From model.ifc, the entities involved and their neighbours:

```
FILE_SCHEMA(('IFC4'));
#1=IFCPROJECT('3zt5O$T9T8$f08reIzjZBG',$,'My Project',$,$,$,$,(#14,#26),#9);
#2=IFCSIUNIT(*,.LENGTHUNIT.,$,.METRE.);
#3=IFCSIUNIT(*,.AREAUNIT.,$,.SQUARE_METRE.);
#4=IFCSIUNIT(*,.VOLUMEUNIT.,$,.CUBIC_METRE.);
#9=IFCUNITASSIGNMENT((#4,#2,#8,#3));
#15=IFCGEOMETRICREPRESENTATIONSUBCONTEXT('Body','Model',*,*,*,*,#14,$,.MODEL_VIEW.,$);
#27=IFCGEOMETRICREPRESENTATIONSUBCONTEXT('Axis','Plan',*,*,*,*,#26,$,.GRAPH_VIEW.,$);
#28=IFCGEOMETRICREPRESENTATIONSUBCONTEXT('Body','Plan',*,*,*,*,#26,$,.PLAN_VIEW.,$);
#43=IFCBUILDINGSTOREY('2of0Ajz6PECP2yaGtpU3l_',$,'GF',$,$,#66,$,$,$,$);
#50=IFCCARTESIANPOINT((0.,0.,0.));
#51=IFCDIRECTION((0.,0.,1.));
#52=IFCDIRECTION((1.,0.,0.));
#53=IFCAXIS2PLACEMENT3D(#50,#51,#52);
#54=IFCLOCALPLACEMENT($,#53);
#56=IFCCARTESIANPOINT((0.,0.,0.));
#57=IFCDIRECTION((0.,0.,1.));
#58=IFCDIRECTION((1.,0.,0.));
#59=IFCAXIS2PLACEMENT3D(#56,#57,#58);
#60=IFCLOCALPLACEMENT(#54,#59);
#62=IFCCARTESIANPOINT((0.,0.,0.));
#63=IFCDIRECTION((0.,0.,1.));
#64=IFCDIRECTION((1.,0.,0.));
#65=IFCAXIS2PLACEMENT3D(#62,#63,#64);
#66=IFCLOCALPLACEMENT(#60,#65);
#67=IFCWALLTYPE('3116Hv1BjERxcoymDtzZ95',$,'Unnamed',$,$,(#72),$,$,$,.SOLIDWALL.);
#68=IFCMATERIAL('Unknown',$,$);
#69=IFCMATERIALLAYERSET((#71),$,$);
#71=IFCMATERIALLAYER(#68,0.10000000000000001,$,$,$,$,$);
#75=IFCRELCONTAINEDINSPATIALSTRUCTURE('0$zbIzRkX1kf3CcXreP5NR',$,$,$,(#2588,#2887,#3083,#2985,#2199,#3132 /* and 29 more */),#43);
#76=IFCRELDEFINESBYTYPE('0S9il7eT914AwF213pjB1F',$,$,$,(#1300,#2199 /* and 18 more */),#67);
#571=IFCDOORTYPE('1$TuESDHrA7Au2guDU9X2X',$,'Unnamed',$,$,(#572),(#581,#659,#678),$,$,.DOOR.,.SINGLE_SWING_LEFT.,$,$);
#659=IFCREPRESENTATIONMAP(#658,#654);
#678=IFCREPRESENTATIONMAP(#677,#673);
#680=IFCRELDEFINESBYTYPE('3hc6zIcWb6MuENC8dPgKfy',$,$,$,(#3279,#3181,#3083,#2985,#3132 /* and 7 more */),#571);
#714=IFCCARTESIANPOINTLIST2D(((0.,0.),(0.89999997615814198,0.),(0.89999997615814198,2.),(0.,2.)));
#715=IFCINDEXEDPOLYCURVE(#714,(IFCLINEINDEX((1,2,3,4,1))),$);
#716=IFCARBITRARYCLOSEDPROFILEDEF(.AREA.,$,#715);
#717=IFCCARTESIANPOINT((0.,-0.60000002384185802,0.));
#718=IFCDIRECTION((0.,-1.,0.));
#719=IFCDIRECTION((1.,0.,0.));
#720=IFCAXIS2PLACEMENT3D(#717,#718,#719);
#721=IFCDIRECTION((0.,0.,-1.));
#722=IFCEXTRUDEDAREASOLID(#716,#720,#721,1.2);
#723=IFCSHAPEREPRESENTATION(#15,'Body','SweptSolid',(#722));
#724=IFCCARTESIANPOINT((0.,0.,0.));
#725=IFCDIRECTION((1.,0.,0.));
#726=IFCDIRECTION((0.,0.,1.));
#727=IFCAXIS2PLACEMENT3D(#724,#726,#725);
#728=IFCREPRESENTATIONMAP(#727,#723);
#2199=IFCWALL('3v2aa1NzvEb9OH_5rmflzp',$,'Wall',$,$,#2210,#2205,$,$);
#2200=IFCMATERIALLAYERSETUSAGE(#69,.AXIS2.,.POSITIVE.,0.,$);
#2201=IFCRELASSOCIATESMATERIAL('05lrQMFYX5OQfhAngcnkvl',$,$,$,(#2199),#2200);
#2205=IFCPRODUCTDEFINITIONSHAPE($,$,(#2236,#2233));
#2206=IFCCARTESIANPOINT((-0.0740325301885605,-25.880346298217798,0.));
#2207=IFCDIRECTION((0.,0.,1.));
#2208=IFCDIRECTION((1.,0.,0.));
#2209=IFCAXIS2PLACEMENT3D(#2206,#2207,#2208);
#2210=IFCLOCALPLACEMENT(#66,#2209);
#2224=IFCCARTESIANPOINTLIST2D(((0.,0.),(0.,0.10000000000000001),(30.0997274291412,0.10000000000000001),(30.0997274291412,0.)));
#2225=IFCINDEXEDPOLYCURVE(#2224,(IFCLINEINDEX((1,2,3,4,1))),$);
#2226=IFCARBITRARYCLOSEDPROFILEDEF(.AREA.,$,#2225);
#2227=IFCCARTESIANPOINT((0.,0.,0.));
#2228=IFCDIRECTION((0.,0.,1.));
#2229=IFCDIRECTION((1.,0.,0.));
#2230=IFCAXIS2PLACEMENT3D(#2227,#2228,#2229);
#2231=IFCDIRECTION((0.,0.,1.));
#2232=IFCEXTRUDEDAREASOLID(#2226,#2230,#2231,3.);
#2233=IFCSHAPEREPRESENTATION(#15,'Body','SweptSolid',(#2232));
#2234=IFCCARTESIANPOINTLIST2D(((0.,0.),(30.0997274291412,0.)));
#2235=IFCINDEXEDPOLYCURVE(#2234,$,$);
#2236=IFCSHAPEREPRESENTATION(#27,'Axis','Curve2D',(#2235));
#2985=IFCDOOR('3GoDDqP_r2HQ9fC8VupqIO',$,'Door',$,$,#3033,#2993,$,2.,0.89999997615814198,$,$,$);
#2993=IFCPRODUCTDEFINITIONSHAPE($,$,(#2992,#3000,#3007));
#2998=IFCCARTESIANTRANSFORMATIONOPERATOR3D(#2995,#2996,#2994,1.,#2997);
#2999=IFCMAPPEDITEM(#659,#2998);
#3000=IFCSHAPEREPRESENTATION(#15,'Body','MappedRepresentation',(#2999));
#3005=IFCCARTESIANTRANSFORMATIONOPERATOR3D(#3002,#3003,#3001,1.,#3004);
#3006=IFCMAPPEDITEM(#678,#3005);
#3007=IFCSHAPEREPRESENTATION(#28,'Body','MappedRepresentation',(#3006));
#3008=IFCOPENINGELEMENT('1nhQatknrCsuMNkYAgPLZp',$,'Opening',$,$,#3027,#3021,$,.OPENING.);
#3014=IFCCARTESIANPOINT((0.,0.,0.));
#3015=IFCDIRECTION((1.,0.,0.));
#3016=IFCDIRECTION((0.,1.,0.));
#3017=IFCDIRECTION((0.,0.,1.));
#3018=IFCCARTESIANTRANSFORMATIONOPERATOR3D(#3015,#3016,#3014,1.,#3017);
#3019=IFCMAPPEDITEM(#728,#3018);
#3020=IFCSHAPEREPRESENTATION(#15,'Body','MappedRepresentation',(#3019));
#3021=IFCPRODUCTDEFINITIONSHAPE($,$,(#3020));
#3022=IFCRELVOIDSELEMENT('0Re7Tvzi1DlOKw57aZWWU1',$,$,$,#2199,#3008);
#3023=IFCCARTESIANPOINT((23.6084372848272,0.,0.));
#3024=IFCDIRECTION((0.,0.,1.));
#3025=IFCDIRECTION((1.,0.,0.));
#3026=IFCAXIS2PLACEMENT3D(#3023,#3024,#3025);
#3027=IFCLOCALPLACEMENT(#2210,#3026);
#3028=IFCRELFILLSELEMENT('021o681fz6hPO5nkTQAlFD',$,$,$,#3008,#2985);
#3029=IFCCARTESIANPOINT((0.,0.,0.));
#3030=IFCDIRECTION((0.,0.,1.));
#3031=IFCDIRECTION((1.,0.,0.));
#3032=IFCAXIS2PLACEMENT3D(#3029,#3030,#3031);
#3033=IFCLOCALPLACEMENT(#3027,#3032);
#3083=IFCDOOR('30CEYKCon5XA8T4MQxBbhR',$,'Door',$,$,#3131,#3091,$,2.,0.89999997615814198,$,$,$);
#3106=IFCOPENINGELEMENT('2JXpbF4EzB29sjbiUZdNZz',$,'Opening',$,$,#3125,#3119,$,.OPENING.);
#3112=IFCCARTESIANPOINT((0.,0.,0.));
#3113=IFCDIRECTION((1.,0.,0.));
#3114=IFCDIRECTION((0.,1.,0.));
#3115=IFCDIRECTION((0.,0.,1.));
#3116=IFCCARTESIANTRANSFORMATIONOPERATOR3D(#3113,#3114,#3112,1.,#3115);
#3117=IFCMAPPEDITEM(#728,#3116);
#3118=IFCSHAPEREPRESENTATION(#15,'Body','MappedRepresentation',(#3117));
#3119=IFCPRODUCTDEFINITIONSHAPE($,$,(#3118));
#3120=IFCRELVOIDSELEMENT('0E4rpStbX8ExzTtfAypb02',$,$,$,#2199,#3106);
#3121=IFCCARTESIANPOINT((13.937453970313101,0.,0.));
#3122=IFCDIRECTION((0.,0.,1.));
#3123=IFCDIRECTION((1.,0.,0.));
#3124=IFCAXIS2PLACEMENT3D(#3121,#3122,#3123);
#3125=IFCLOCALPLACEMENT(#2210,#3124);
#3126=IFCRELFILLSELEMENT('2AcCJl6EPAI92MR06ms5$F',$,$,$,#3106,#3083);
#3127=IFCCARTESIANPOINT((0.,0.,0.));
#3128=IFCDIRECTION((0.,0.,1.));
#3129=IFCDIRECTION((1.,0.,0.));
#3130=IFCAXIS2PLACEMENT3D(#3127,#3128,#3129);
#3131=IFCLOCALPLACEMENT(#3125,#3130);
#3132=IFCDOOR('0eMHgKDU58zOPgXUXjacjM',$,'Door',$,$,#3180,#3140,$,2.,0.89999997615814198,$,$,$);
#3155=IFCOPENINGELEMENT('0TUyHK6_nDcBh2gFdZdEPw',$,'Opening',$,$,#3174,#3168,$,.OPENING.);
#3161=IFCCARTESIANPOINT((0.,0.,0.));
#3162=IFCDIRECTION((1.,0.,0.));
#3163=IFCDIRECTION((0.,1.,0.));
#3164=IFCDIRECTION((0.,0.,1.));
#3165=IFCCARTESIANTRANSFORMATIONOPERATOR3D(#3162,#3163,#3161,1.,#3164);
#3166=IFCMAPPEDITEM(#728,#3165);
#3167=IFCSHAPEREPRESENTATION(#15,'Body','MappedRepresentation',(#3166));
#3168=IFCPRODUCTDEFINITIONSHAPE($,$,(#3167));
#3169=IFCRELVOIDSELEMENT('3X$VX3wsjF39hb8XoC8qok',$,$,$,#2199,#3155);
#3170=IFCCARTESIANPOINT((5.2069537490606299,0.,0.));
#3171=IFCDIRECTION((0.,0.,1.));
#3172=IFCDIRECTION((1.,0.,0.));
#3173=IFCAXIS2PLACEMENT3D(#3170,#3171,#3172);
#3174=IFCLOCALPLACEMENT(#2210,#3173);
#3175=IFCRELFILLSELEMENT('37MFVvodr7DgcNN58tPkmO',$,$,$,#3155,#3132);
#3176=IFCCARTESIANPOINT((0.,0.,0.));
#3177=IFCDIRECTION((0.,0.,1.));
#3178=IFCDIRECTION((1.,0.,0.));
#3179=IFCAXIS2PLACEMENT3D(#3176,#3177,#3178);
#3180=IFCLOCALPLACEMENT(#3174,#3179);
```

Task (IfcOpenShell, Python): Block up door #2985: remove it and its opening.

```python
import ifcopenshell
import ifcopenshell.api.feature
import ifcopenshell.api.root
import ifcopenshell.geom
import ifcopenshell.util.shape

model = ifcopenshell.open("model.ifc")
settings = ifcopenshell.geom.settings()


def volume(element):
    """Net volume in cubic metres, openings subtracted."""
    shape = ifcopenshell.geom.create_shape(settings, element)
    return ifcopenshell.util.shape.get_volume(shape.geometry)


door = model.by_guid("3GoDDqP_r2HQ9fC8VupqIO")
opening = door.FillsVoids[0].RelatingOpeningElement
wall = opening.VoidsElements[0].RelatingBuildingElement
before = volume(wall)

ifcopenshell.api.root.remove_product(model, product=door)
ifcopenshell.api.feature.remove_feature(model, feature=opening)

after = volume(wall)

print(f"wall volume {before:.3f} -> {after:.3f} m3")

model.write("model_v2.ifc")
```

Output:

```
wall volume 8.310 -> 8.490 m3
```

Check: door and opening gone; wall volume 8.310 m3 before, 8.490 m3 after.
